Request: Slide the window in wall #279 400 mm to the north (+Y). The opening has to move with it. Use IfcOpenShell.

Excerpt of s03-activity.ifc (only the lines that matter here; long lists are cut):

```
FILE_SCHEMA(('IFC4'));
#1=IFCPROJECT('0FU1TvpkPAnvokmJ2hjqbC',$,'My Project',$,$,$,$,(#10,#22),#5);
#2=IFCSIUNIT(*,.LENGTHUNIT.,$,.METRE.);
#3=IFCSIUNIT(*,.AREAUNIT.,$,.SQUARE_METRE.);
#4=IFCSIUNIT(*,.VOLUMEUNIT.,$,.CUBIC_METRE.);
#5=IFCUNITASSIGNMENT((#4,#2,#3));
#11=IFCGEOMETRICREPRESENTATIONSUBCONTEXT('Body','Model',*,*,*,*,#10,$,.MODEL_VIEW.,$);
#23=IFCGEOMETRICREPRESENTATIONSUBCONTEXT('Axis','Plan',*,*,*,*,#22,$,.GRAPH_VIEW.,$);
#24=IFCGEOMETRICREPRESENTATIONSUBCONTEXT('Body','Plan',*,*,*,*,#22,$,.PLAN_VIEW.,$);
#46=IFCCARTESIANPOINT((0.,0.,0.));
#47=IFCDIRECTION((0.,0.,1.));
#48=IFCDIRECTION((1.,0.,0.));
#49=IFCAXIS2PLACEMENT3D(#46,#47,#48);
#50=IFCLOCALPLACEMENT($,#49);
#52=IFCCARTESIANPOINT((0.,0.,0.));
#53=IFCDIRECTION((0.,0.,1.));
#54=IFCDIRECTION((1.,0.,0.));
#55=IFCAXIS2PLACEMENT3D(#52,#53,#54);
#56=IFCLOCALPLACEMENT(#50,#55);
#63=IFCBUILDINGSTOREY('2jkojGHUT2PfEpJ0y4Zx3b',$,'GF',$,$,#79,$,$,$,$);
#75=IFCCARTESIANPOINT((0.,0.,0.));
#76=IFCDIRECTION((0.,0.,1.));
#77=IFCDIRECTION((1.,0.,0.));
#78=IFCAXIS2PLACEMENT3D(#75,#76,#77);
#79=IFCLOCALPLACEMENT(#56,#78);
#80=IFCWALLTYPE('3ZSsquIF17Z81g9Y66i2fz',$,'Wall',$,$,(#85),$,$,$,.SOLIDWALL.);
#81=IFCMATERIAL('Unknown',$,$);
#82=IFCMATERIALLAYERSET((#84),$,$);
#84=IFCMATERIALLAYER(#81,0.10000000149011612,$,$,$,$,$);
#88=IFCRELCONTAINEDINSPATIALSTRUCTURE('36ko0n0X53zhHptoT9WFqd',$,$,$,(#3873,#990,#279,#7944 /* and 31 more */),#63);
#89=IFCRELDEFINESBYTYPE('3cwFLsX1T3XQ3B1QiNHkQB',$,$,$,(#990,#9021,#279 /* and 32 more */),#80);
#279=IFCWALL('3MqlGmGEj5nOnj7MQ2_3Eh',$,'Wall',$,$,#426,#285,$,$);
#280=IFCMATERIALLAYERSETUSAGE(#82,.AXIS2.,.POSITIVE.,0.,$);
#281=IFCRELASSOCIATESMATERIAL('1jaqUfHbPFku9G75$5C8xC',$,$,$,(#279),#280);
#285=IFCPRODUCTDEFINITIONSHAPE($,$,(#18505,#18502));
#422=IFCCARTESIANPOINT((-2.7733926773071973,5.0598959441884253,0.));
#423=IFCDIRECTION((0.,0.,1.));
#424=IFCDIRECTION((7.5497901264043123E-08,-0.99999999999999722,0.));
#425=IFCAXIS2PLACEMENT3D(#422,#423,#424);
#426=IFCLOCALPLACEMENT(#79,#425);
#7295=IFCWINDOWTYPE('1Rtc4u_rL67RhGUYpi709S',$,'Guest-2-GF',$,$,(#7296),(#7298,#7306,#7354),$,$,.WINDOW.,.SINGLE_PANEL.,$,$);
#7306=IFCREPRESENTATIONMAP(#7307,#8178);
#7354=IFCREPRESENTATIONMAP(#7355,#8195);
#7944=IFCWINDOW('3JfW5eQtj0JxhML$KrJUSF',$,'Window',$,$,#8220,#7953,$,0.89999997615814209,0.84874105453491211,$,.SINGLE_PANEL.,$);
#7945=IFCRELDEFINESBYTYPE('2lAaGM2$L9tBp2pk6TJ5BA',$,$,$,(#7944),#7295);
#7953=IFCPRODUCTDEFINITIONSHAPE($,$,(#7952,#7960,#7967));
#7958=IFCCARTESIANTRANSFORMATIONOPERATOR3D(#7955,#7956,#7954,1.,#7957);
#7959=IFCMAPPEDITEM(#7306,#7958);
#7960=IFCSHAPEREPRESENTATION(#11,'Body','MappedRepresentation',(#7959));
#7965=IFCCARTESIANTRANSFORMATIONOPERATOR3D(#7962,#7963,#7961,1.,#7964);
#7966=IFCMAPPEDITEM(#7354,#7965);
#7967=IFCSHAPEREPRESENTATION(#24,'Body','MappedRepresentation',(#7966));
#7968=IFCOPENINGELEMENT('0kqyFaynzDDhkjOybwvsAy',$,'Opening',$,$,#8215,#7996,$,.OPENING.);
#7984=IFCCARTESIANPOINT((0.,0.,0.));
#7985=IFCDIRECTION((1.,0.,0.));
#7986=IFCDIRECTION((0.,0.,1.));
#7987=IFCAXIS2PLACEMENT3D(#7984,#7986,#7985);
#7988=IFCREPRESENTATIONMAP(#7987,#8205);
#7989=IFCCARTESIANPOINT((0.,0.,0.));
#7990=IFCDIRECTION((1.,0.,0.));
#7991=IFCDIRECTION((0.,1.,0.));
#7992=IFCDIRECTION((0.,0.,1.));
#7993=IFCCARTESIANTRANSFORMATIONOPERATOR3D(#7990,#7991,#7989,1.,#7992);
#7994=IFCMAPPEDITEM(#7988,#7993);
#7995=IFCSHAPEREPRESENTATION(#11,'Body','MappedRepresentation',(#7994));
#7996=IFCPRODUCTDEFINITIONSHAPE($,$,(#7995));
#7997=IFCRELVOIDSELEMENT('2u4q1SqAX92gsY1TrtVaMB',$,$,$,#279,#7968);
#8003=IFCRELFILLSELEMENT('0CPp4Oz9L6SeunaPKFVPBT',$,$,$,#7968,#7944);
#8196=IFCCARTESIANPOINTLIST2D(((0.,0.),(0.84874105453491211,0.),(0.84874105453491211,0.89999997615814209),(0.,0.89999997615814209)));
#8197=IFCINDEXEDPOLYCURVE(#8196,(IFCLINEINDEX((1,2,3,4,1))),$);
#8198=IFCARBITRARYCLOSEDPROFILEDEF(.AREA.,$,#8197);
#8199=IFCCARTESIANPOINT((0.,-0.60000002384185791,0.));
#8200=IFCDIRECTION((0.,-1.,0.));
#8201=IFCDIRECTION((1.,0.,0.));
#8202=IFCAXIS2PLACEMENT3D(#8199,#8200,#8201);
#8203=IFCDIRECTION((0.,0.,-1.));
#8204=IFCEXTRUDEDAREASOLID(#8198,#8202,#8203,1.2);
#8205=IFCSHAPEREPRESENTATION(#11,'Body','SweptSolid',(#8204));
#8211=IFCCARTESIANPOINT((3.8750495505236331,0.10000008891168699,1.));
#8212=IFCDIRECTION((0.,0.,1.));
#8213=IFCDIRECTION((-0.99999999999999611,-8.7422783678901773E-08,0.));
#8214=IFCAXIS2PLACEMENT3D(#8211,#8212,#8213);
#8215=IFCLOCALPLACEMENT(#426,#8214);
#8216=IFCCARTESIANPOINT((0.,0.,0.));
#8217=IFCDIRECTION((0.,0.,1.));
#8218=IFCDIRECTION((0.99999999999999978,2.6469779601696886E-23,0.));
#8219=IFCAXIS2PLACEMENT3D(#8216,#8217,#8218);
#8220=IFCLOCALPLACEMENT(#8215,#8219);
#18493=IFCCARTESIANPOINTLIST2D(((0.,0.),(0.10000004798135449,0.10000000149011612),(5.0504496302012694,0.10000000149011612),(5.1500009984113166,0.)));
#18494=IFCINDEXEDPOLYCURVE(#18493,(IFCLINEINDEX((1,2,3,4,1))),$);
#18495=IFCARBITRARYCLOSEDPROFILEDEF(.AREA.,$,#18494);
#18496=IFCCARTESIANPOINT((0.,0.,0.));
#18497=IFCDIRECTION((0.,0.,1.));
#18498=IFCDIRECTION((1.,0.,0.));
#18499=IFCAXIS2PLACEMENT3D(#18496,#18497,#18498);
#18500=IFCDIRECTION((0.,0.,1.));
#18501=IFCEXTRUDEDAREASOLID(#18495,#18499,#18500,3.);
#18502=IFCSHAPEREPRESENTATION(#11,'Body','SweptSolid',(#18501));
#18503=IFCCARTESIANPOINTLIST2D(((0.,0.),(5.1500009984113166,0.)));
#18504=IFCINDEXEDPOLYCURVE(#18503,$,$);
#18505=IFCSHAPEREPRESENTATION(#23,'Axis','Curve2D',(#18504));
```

```python
import ifcopenshell
import ifcopenshell.api.geometry
import ifcopenshell.util.placement
import ifcopenshell.util.unit

model = ifcopenshell.open("s03-activity.ifc")
unit_scale = ifcopenshell.util.unit.calculate_unit_scale(model)

window = model.by_id(7944)
opening = window.FillsVoids[0].RelatingOpeningElement
wall = opening.VoidsElements[0].RelatingBuildingElement

wall_matrix = ifcopenshell.util.placement.get_local_placement(wall.ObjectPlacement)
shift = wall_matrix[:3, 0] * -0.4 / unit_scale
before = ifcopenshell.util.placement.get_local_placement(window.ObjectPlacement)[:3, 3].copy()

# The window is placed relative to its opening, so it follows when the opening moves.
matrix = ifcopenshell.util.placement.get_local_placement(opening.ObjectPlacement)
matrix[:3, 3] += shift
ifcopenshell.api.geometry.edit_object_placement(
    model, product=opening, matrix=matrix, is_si=False, should_transform_children=True
)

after = ifcopenshell.util.placement.get_local_placement(window.ObjectPlacement)[:3, 3]
print("window moved by", (after - before).round(3) + 0.0)

model.write("s03-activity_updated.ifc")
```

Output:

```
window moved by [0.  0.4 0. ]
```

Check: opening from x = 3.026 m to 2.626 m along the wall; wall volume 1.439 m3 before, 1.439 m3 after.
